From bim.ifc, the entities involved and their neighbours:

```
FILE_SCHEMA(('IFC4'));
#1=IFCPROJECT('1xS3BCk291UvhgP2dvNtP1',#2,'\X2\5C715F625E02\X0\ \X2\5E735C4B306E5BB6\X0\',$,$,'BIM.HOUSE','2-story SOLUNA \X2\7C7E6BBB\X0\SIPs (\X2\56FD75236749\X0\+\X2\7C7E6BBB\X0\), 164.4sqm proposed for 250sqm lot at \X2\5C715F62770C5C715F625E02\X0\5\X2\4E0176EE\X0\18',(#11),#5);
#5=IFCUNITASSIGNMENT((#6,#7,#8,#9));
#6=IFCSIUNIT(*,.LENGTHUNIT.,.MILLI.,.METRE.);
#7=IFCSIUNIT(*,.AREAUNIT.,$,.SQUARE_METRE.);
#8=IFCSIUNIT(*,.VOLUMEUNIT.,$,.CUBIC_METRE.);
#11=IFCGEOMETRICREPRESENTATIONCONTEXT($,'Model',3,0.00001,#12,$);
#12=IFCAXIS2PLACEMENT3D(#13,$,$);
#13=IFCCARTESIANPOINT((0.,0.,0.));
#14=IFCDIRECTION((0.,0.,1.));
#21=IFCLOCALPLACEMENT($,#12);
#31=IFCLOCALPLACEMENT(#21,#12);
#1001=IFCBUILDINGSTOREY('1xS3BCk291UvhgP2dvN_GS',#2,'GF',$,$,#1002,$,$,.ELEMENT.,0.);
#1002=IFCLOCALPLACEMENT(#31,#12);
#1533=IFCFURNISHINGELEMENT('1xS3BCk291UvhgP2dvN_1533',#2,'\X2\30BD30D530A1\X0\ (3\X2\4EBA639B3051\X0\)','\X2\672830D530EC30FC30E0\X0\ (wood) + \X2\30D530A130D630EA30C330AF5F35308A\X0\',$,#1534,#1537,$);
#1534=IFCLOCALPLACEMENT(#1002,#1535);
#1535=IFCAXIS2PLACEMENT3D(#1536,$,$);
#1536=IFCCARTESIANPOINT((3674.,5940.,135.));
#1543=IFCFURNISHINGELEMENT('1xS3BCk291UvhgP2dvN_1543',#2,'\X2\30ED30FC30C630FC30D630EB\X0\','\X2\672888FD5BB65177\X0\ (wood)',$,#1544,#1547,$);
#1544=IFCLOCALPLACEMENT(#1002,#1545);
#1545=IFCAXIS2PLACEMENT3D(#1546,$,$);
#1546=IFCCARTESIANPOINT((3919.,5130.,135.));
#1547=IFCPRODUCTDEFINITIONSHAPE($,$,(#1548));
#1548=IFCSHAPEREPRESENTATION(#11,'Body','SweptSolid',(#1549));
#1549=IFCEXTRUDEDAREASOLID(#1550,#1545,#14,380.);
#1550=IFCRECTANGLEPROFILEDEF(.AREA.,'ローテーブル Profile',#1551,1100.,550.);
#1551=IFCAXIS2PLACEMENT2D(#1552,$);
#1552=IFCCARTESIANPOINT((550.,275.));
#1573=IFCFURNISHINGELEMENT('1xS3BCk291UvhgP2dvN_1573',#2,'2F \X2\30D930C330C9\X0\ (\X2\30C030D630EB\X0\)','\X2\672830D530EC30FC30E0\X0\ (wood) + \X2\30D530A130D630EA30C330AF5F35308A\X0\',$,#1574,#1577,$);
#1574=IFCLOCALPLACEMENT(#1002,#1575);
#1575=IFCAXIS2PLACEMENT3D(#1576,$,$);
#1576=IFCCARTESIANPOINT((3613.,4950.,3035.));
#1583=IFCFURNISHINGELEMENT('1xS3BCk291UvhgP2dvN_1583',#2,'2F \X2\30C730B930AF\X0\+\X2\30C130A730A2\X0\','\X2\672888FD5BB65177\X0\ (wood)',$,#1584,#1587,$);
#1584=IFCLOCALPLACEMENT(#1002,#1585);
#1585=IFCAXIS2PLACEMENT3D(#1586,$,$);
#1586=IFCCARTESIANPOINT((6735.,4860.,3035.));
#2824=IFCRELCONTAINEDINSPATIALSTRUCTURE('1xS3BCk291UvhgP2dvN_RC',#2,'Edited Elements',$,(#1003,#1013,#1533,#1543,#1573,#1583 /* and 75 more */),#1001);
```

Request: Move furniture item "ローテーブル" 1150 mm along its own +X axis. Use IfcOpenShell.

```python
import ifcopenshell
import ifcopenshell.api.geometry
import ifcopenshell.util.placement
import ifcopenshell.util.unit

model = ifcopenshell.open("bim.ifc")
unit_scale = ifcopenshell.util.unit.calculate_unit_scale(model)

item = model.by_id(1543)
matrix = ifcopenshell.util.placement.get_local_placement(item.ObjectPlacement)
matrix[:3, 3] += matrix[:3, 0] * 1.15 / unit_scale
ifcopenshell.api.geometry.edit_object_placement(model, product=item, matrix=matrix, is_si=False)

print(ifcopenshell.util.placement.get_local_placement(item.ObjectPlacement).round(3) + 0.0)

model.write("bim_updated.ifc")
```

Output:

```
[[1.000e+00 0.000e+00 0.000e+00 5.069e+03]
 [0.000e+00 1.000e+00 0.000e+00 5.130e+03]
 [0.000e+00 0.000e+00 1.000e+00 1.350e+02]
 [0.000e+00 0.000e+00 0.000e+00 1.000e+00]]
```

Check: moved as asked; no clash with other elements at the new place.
